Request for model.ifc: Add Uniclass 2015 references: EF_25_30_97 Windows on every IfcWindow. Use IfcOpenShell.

First a look at what the model holds.

```python
import ifcopenshell

model = ifcopenshell.open("model.ifc")
print(model.schema)
print("classifications:", [c.Name for c in model.by_type("IfcClassification")])
for ifc_class in ("IfcDoor", "IfcRoof", "IfcStair", "IfcWall", "IfcWindow"):
    print(ifc_class, len(model.by_type(ifc_class)))
```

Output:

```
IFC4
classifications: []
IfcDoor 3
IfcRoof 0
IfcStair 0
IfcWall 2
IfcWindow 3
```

```python
import ifcopenshell
import ifcopenshell.api.classification

model = ifcopenshell.open("model.ifc")

system = ifcopenshell.api.classification.add_classification(model, classification="Uniclass 2015")

codes = {
    "IfcWindow": ("EF_25_30_97", "Windows"),
}
for ifc_class, (code, name) in codes.items():
    products = model.by_type(ifc_class)
    ifcopenshell.api.classification.add_reference(
        model, products=products, classification=system, identification=code, name=name
    )
    print(code, len(products))

model.write("model_v2.ifc")
```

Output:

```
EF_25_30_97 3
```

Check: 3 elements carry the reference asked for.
